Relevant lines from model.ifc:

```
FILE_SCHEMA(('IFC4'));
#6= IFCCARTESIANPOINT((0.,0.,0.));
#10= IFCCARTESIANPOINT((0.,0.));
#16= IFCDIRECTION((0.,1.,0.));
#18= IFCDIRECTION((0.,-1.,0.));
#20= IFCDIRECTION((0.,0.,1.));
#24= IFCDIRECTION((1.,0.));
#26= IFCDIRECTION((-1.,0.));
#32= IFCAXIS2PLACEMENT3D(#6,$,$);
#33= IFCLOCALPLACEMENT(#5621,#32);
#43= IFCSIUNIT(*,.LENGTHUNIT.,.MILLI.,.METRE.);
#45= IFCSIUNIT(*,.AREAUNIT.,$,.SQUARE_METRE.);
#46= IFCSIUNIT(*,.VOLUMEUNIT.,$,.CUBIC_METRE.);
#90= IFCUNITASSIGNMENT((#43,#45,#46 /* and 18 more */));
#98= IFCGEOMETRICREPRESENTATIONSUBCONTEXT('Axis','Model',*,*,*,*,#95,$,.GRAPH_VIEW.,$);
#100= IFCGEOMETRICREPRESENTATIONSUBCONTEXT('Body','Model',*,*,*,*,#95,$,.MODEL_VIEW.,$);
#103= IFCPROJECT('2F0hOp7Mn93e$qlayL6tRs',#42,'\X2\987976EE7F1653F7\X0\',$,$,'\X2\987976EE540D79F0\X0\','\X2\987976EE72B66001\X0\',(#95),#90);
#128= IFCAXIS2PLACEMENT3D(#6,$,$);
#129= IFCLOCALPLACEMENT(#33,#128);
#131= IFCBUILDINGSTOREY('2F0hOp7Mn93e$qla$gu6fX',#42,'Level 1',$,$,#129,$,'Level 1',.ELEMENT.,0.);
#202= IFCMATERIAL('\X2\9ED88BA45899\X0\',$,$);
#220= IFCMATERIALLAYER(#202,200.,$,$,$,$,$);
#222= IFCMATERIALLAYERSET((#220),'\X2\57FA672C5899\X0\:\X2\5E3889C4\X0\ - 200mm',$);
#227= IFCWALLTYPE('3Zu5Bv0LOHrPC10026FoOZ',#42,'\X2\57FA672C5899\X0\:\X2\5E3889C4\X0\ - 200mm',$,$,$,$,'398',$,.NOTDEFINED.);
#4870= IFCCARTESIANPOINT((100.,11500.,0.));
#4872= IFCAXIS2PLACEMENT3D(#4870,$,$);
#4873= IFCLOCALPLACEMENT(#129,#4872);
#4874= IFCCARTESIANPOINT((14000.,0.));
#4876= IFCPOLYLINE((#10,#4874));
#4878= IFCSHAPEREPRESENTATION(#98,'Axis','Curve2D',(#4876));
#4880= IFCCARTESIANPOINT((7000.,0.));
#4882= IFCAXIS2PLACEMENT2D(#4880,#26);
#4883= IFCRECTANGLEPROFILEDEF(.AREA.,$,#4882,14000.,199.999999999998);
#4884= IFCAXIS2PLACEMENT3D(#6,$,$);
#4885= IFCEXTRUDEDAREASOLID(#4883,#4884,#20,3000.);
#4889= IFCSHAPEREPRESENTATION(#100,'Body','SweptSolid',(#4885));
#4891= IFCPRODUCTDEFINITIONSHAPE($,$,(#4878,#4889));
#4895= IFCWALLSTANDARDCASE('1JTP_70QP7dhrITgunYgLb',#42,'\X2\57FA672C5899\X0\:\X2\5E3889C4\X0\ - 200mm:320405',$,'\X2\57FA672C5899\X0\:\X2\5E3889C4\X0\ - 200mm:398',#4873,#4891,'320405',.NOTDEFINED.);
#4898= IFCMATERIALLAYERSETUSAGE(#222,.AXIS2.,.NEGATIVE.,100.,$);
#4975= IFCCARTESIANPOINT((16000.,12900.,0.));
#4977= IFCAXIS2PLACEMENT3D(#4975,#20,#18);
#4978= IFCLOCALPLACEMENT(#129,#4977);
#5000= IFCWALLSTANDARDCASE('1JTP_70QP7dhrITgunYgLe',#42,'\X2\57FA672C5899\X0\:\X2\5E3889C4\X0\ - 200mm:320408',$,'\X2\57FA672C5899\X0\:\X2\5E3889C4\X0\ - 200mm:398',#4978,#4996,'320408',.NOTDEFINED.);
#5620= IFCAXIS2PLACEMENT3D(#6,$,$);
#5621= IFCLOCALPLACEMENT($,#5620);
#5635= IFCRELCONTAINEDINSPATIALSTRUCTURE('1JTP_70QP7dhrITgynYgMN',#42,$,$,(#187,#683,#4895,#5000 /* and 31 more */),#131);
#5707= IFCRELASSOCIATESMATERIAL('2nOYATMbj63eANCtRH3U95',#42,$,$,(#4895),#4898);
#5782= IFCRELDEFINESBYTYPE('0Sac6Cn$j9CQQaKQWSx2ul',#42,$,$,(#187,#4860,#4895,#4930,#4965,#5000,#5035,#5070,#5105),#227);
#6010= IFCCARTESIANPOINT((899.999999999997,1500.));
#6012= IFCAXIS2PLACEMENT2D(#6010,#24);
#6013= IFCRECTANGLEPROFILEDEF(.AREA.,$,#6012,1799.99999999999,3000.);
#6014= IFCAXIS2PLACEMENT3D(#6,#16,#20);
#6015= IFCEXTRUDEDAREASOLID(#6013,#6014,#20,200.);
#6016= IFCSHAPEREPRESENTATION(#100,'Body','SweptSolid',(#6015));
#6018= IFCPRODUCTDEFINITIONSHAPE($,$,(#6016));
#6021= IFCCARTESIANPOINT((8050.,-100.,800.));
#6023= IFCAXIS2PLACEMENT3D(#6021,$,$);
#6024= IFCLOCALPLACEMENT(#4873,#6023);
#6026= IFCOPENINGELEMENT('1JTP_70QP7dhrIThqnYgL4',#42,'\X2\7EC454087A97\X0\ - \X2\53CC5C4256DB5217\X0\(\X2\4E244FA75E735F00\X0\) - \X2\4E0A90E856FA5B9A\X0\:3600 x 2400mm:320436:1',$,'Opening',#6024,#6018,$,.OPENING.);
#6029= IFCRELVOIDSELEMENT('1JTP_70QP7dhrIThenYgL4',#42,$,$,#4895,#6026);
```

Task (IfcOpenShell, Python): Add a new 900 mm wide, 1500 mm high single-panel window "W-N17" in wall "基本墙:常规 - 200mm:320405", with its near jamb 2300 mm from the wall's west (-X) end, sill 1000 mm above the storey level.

```python
import numpy as np
import ifcopenshell
import ifcopenshell.api.feature
import ifcopenshell.api.geometry
import ifcopenshell.api.root
import ifcopenshell.api.spatial
import ifcopenshell.geom
import ifcopenshell.util.element
import ifcopenshell.util.placement
import ifcopenshell.util.representation
import ifcopenshell.util.shape
import ifcopenshell.util.unit

model = ifcopenshell.open("model.ifc")
unit_scale = ifcopenshell.util.unit.calculate_unit_scale(model)
settings = ifcopenshell.geom.settings()


def volume(element):
    """Net volume in cubic metres, openings subtracted."""
    shape = ifcopenshell.geom.create_shape(settings, element)
    return ifcopenshell.util.shape.get_volume(shape.geometry)


wall = model.by_guid("1JTP_70QP7dhrITgunYgLb")
storey = ifcopenshell.util.element.get_container(wall, ifc_class="IfcBuildingStorey")
context = ifcopenshell.util.representation.get_context(model, "Model", "Body", "MODEL_VIEW")
before = volume(wall)

width, height, from_end, sill = 0.9, 1.5, 2.3, 1  # metres

# The wall runs along its own X axis, and the end named is its -X end.
wall_shape = ifcopenshell.geom.create_shape(settings, wall)
x, y, z = ifcopenshell.util.shape.get_vertices(wall_shape.geometry).T
start = x.min() + from_end
face, thickness = float(y.min()), float(y.max() - y.min())
wall_matrix = ifcopenshell.util.placement.get_local_placement(wall.ObjectPlacement)
level = ifcopenshell.util.placement.get_local_placement(storey.ObjectPlacement)[2, 3]


def in_wall(x, y):
    """Placement at x, y metres in the wall's axes, at sill height."""
    matrix = wall_matrix.copy()
    matrix[:, 3] = wall_matrix @ np.array([x / unit_scale, y / unit_scale, 0.0, 1.0])
    matrix[2, 3] = level + sill / unit_scale
    return matrix


# Opening: a box that overshoots both wall faces by 50 mm.
opening = ifcopenshell.api.root.create_entity(model, ifc_class="IfcOpeningElement", predefined_type="OPENING")
box = ifcopenshell.api.geometry.add_wall_representation(
    model, context=context, length=width, height=height, thickness=thickness + 0.1
)
ifcopenshell.api.geometry.assign_representation(model, product=opening, representation=box)
ifcopenshell.api.geometry.edit_object_placement(model, product=opening, matrix=in_wall(start, face - 0.05), is_si=False)
ifcopenshell.api.feature.add_feature(model, feature=opening, element=wall)

window = ifcopenshell.api.root.create_entity(model, ifc_class="IfcWindow", name="W-N17", predefined_type="WINDOW")
window.OverallWidth, window.OverallHeight = width / unit_scale, height / unit_scale
window.PartitioningType = "SINGLE_PANEL"
body = ifcopenshell.api.geometry.add_window_representation(
    model,
    context=context,
    overall_width=window.OverallWidth,
    overall_height=window.OverallHeight,
    partition_type="SINGLE_PANEL",
)
ifcopenshell.api.geometry.assign_representation(model, product=window, representation=body)
ifcopenshell.api.spatial.assign_container(model, products=[window], relating_structure=storey)
ifcopenshell.api.feature.add_filling(model, opening=opening, element=window)

# Centre the window in the wall's thickness.
ifcopenshell.api.geometry.edit_object_placement(model, product=window, matrix=in_wall(start, face), is_si=False)
window_shape = ifcopenshell.geom.create_shape(settings, window)
depth = ifcopenshell.util.shape.get_vertices(window_shape.geometry)[:, 1]
offset = face + thickness / 2 - (depth.min() + depth.max()) / 2
ifcopenshell.api.geometry.edit_object_placement(model, product=window, matrix=in_wall(start, offset), is_si=False)

after = volume(wall)

print(f"wall volume {before:.3f} -> {after:.3f} m3")

model.write("model-out.ifc")
```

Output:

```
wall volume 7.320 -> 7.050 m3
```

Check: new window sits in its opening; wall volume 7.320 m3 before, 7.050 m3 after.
